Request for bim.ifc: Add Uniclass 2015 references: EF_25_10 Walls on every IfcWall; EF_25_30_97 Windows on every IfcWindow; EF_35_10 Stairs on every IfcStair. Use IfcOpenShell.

First a look at what the model holds.

```python
import ifcopenshell

model = ifcopenshell.open("bim.ifc")
print(model.schema)
print("classifications:", [c.Name for c in model.by_type("IfcClassification")])
for ifc_class in ("IfcDoor", "IfcRoof", "IfcStair", "IfcWall", "IfcWindow"):
    print(ifc_class, len(model.by_type(ifc_class)))
```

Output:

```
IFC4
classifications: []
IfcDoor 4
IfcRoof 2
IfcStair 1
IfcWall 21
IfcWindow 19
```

```python
import ifcopenshell
import ifcopenshell.api.classification

model = ifcopenshell.open("bim.ifc")

system = ifcopenshell.api.classification.add_classification(model, classification="Uniclass 2015")

codes = {
    "IfcWall": ("EF_25_10", "Walls"),
    "IfcWindow": ("EF_25_30_97", "Windows"),
    "IfcStair": ("EF_35_10", "Stairs"),
}
for ifc_class, (code, name) in codes.items():
    products = model.by_type(ifc_class)
    ifcopenshell.api.classification.add_reference(
        model, products=products, classification=system, identification=code, name=name
    )
    print(code, len(products))

model.write("bim_v2.ifc")
```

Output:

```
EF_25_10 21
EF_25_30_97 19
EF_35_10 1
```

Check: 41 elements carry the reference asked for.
